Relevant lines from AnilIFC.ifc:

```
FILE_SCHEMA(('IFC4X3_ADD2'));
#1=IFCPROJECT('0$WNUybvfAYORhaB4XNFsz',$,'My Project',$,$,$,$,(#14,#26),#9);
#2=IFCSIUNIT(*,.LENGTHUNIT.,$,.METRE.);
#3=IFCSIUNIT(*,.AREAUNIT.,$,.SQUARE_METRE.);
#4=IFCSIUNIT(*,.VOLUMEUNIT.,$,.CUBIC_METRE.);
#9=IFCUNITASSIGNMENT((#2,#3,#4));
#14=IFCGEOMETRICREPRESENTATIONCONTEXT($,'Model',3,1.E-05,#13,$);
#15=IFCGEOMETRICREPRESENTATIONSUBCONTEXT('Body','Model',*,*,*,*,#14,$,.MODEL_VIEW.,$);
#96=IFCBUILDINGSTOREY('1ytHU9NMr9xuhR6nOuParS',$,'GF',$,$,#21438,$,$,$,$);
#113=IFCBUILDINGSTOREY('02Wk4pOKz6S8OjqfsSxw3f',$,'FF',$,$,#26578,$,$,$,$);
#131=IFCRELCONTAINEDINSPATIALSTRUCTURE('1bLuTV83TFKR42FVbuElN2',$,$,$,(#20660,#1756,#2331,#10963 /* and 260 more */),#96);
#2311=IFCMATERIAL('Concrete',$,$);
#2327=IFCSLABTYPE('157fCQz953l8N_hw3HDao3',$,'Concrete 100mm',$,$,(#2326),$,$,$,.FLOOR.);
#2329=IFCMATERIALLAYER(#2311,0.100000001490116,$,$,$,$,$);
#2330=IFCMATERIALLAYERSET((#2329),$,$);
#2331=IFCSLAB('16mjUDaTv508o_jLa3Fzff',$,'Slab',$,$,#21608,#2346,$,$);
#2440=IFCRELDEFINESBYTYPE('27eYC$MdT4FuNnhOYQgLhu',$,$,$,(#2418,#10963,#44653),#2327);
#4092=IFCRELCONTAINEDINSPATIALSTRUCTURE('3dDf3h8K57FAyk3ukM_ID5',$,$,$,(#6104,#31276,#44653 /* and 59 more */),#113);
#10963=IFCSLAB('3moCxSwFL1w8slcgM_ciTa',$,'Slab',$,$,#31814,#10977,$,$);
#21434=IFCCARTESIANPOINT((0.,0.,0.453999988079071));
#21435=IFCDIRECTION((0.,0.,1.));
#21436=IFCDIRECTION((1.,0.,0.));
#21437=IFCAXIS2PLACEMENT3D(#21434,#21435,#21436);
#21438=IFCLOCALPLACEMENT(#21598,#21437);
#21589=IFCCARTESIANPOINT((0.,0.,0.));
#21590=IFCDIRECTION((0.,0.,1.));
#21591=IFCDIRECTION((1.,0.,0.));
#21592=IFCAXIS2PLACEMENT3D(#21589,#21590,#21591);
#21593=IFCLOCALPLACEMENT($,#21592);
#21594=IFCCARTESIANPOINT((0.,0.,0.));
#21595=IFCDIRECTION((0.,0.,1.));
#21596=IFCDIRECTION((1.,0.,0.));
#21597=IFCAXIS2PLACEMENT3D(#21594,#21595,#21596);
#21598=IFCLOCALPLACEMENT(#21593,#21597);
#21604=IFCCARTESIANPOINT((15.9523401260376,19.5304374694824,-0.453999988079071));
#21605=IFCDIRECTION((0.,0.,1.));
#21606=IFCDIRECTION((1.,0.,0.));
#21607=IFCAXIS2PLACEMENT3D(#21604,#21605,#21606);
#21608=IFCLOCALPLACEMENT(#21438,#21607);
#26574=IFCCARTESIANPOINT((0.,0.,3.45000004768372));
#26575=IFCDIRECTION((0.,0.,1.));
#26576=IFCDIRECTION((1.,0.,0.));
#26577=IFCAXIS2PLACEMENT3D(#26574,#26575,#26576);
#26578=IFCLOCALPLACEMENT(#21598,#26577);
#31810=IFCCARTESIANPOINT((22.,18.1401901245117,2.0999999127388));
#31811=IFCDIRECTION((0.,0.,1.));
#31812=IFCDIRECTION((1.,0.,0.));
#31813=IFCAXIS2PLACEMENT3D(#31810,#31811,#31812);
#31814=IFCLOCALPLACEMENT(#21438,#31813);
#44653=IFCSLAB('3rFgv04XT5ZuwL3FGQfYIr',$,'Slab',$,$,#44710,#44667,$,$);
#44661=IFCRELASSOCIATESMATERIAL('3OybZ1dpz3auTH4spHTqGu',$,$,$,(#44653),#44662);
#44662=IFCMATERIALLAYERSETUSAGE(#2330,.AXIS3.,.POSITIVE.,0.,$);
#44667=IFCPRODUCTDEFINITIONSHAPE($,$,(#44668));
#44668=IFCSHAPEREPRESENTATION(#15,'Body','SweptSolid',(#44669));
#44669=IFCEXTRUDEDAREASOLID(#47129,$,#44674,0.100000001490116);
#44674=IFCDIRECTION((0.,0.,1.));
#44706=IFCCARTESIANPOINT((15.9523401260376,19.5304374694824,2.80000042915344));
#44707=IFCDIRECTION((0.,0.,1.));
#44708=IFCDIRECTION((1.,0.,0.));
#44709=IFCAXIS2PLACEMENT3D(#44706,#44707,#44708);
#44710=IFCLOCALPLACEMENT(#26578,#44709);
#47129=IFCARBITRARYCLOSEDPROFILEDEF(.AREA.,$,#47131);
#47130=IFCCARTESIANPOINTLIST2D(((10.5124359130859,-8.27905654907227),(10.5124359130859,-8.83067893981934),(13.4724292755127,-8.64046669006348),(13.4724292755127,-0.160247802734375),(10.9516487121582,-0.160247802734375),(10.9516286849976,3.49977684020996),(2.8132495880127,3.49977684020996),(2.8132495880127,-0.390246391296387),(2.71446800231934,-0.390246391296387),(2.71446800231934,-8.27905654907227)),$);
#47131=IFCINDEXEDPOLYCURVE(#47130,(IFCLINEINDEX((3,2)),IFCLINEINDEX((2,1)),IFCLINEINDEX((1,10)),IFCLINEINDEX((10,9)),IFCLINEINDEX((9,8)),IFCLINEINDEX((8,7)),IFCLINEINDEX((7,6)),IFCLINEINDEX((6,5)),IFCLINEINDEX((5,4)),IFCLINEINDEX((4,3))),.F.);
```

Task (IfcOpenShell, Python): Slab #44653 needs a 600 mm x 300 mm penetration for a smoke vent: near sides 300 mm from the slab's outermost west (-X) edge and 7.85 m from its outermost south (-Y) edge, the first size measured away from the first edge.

```python
import numpy as np
import ifcopenshell
import ifcopenshell.api.feature
import ifcopenshell.api.geometry
import ifcopenshell.api.root
import ifcopenshell.geom
import ifcopenshell.util.placement
import ifcopenshell.util.representation
import ifcopenshell.util.shape
import ifcopenshell.util.unit

model = ifcopenshell.open("AnilIFC.ifc")
unit_scale = ifcopenshell.util.unit.calculate_unit_scale(model)
settings = ifcopenshell.geom.settings()


def volume(element):
    """Net volume in cubic metres, openings subtracted."""
    shape = ifcopenshell.geom.create_shape(settings, element)
    return ifcopenshell.util.shape.get_volume(shape.geometry)


slab = model.by_guid("3rFgv04XT5ZuwL3FGQfYIr")
before = volume(slab)

# Extent in the slab's own axes, in metres. The edges named are its -X and -Y sides.
slab_shape = ifcopenshell.geom.create_shape(settings, slab)
vertices = ifcopenshell.util.shape.get_vertices(slab_shape.geometry)
x_min, y_min, bottom = vertices.min(axis=0)
top = vertices[:, 2].max()

opening = ifcopenshell.api.root.create_entity(model, ifc_class="IfcOpeningElement", name="Smoke vent opening", predefined_type="OPENING")
context = ifcopenshell.util.representation.get_context(model, "Model", "Body", "MODEL_VIEW")
width, depth = 0.6, 0.3
outline = [(0.0, 0.0), (width, 0.0), (width, depth), (0.0, depth), (0.0, 0.0)]
# Overshoot both faces by 50 mm so the cut is clean.
shape = ifcopenshell.api.geometry.add_slab_representation(
    model, context=context, depth=top - bottom + 0.1, polyline=outline
)
ifcopenshell.api.geometry.assign_representation(model, product=opening, representation=shape)

matrix = ifcopenshell.util.placement.get_local_placement(slab.ObjectPlacement)
matrix[:, 3] = matrix @ np.append(np.array([x_min + 0.3, y_min + 7.85, bottom - 0.05]) / unit_scale, 1.0)
ifcopenshell.api.geometry.edit_object_placement(model, product=opening, matrix=matrix, is_si=False)
ifcopenshell.api.feature.add_feature(model, feature=opening, element=slab)

after = volume(slab)

print(f"slab volume {before:.3f} -> {after:.3f} m3")

model.write("AnilIFC_edited.ifc")
```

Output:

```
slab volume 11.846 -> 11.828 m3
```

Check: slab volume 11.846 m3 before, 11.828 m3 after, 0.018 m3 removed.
